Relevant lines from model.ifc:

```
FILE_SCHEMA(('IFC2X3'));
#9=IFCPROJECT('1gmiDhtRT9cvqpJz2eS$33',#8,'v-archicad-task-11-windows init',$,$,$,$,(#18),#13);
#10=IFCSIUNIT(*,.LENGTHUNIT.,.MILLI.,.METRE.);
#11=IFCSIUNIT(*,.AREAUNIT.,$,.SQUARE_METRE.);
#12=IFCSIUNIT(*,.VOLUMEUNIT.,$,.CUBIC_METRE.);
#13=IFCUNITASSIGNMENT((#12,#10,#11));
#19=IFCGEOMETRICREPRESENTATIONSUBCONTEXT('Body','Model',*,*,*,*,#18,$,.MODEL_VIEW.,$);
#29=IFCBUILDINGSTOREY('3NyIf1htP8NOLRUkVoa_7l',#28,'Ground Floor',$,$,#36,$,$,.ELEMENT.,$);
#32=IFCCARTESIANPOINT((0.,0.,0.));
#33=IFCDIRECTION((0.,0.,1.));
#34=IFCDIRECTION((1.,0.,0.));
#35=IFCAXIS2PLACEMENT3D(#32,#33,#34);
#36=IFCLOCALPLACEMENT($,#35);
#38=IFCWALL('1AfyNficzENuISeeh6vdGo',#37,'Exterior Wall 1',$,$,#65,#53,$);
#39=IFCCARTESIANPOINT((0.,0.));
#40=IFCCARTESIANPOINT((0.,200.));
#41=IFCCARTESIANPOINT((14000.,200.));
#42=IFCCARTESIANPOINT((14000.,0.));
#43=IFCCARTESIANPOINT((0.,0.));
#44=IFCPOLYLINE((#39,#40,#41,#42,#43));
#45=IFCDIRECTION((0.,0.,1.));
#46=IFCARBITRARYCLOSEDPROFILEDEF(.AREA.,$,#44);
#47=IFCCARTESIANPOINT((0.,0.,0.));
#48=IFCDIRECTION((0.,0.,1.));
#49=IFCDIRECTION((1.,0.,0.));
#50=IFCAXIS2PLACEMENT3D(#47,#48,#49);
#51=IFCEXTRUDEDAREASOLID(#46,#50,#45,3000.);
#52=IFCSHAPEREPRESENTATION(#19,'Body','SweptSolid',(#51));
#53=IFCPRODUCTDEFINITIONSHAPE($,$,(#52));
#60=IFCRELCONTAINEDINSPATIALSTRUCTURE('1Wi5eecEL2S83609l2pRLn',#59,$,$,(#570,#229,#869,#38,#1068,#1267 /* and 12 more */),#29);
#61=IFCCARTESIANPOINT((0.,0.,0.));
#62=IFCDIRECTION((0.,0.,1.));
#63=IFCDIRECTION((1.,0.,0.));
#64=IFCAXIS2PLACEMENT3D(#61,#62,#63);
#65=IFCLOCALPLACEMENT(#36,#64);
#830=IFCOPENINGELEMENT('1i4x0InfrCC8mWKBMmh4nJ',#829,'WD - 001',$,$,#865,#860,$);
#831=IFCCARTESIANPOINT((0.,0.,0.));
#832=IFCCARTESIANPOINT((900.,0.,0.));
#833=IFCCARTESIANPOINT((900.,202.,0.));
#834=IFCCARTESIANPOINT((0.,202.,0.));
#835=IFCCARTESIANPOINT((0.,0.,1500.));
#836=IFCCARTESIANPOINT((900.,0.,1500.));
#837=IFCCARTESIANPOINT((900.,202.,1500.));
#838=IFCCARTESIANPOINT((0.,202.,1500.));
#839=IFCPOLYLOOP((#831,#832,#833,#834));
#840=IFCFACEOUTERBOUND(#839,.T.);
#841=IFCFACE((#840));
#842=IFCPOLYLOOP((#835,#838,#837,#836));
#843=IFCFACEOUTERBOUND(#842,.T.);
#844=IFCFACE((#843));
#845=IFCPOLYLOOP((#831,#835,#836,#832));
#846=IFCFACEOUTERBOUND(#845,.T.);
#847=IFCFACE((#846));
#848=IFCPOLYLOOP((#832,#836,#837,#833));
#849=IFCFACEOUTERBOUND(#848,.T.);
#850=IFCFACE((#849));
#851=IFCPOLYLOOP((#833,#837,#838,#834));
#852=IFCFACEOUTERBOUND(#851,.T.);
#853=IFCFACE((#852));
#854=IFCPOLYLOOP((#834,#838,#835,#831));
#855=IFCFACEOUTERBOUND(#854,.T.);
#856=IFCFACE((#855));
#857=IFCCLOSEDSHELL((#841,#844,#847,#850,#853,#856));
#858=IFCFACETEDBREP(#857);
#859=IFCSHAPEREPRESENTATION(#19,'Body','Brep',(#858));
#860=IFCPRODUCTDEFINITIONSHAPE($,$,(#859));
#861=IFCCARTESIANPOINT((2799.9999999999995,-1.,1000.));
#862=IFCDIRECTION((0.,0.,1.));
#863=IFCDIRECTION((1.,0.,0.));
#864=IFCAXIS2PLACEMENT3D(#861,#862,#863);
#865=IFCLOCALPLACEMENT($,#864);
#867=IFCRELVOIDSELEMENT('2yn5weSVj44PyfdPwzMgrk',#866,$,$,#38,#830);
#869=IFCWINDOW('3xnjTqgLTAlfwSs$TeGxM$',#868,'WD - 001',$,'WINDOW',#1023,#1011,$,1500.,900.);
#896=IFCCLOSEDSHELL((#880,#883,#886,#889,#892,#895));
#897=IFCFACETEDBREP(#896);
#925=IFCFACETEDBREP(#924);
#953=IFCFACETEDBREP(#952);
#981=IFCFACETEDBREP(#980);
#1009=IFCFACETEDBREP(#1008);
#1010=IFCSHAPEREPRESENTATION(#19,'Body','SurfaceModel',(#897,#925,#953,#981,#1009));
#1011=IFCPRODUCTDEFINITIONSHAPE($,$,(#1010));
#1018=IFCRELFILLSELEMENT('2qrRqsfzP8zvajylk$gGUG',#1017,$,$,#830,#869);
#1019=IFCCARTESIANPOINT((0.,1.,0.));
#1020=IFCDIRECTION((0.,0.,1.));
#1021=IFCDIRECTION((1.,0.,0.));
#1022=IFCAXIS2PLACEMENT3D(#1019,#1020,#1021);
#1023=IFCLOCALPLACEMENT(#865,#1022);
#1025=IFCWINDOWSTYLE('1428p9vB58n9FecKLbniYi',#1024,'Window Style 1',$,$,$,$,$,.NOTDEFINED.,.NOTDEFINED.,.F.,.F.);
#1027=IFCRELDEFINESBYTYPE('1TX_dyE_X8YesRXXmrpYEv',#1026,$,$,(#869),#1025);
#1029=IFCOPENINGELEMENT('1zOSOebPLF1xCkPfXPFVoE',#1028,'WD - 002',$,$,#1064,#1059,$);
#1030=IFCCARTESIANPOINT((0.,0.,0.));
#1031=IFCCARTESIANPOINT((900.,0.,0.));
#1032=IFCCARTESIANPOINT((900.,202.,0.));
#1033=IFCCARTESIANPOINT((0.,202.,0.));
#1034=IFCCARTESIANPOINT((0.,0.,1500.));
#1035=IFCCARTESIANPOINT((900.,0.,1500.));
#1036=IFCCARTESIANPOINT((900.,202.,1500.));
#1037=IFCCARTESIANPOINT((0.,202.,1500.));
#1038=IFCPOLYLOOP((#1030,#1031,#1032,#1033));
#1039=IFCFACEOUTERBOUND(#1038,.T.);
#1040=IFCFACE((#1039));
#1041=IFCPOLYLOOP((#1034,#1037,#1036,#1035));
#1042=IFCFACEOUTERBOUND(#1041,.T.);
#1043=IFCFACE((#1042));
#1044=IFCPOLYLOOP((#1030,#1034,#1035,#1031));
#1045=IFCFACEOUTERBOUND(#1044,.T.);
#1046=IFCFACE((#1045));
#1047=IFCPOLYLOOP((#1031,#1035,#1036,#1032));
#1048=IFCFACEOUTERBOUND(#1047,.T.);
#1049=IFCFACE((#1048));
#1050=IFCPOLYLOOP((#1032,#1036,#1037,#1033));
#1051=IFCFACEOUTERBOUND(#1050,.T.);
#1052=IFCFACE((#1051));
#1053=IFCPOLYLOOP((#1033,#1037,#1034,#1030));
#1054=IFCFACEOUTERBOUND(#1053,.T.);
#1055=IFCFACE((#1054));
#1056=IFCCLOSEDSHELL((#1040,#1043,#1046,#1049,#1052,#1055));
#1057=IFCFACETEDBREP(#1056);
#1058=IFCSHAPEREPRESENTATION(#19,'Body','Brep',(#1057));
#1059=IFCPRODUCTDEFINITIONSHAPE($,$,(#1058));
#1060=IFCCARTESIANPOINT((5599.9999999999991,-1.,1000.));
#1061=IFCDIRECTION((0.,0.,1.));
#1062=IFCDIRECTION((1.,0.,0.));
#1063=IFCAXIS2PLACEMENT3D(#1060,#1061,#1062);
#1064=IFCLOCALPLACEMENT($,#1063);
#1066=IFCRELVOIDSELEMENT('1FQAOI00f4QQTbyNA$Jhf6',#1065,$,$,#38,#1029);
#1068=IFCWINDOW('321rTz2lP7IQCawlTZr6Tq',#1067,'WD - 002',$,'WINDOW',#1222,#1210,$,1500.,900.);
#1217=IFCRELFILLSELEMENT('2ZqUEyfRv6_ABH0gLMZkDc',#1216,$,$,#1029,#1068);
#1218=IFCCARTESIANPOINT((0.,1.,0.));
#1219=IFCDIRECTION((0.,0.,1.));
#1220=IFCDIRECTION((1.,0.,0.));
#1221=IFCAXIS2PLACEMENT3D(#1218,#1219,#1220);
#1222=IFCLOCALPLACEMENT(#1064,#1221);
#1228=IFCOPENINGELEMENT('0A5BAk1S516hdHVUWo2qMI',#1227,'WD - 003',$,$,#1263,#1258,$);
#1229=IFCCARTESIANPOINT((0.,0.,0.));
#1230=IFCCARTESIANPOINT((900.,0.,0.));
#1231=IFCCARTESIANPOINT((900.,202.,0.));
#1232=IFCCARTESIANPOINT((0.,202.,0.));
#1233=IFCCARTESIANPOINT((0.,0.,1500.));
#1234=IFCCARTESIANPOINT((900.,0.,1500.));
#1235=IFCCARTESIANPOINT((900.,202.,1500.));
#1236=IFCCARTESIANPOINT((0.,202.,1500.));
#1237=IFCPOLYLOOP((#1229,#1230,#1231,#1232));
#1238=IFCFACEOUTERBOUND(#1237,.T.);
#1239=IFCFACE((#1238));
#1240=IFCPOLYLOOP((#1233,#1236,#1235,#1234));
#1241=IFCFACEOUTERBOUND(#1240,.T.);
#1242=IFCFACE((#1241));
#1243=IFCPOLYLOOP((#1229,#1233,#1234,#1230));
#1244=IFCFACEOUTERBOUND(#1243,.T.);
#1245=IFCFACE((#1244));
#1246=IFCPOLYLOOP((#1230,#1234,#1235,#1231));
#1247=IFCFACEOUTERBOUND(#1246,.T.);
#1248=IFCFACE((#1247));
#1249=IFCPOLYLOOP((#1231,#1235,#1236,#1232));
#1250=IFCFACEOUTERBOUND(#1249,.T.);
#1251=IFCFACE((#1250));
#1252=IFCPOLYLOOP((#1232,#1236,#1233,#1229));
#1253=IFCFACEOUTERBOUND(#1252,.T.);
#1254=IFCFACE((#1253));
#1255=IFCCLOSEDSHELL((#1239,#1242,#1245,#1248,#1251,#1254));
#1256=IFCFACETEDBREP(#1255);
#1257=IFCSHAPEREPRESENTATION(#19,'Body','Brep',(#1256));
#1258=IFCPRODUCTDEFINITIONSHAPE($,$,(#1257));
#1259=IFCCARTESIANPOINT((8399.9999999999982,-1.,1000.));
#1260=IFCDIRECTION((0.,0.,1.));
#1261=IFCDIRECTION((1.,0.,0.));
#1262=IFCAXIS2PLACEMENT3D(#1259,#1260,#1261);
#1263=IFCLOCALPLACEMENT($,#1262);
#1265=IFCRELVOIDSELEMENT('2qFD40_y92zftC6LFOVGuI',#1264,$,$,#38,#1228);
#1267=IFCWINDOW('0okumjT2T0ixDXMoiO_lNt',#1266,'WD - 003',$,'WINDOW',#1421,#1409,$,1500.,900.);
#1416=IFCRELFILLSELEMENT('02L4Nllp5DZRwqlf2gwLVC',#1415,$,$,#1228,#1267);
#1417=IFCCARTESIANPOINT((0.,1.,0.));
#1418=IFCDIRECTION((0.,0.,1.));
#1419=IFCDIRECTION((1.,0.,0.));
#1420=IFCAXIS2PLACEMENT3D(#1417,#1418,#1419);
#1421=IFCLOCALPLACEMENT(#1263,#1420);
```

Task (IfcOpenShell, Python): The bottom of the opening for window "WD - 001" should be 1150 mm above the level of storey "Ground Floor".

```python
import numpy as np
import ifcopenshell
import ifcopenshell.api.geometry
import ifcopenshell.geom
import ifcopenshell.util.element
import ifcopenshell.util.placement
import ifcopenshell.util.shape
import ifcopenshell.util.unit

model = ifcopenshell.open("model.ifc")
unit_scale = ifcopenshell.util.unit.calculate_unit_scale(model)

window = model.by_id(869)
opening = window.FillsVoids[0].RelatingOpeningElement
storey = ifcopenshell.util.element.get_container(window, ifc_class="IfcBuildingStorey")
level = ifcopenshell.util.placement.get_local_placement(storey.ObjectPlacement)[2, 3]

# The opening's origin need not be at the sill, so measure its lowest point.
shape = ifcopenshell.geom.create_shape(ifcopenshell.geom.settings(), opening)
bottom = ifcopenshell.util.shape.get_shape_bottom_elevation(shape, shape.geometry) / unit_scale
dz = level + 1.15 / unit_scale - bottom

shift = np.array([0.0, 0.0, dz])
# The window is placed relative to its opening, so it follows when the opening moves.
matrix = ifcopenshell.util.placement.get_local_placement(opening.ObjectPlacement)
matrix[:3, 3] += shift
ifcopenshell.api.geometry.edit_object_placement(
    model, product=opening, matrix=matrix, is_si=False, should_transform_children=True
)

print(f"moved by {dz * unit_scale:+.3f} m")

model.write("model_edited.ifc")
```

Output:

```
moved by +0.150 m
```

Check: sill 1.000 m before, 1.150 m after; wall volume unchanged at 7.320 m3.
